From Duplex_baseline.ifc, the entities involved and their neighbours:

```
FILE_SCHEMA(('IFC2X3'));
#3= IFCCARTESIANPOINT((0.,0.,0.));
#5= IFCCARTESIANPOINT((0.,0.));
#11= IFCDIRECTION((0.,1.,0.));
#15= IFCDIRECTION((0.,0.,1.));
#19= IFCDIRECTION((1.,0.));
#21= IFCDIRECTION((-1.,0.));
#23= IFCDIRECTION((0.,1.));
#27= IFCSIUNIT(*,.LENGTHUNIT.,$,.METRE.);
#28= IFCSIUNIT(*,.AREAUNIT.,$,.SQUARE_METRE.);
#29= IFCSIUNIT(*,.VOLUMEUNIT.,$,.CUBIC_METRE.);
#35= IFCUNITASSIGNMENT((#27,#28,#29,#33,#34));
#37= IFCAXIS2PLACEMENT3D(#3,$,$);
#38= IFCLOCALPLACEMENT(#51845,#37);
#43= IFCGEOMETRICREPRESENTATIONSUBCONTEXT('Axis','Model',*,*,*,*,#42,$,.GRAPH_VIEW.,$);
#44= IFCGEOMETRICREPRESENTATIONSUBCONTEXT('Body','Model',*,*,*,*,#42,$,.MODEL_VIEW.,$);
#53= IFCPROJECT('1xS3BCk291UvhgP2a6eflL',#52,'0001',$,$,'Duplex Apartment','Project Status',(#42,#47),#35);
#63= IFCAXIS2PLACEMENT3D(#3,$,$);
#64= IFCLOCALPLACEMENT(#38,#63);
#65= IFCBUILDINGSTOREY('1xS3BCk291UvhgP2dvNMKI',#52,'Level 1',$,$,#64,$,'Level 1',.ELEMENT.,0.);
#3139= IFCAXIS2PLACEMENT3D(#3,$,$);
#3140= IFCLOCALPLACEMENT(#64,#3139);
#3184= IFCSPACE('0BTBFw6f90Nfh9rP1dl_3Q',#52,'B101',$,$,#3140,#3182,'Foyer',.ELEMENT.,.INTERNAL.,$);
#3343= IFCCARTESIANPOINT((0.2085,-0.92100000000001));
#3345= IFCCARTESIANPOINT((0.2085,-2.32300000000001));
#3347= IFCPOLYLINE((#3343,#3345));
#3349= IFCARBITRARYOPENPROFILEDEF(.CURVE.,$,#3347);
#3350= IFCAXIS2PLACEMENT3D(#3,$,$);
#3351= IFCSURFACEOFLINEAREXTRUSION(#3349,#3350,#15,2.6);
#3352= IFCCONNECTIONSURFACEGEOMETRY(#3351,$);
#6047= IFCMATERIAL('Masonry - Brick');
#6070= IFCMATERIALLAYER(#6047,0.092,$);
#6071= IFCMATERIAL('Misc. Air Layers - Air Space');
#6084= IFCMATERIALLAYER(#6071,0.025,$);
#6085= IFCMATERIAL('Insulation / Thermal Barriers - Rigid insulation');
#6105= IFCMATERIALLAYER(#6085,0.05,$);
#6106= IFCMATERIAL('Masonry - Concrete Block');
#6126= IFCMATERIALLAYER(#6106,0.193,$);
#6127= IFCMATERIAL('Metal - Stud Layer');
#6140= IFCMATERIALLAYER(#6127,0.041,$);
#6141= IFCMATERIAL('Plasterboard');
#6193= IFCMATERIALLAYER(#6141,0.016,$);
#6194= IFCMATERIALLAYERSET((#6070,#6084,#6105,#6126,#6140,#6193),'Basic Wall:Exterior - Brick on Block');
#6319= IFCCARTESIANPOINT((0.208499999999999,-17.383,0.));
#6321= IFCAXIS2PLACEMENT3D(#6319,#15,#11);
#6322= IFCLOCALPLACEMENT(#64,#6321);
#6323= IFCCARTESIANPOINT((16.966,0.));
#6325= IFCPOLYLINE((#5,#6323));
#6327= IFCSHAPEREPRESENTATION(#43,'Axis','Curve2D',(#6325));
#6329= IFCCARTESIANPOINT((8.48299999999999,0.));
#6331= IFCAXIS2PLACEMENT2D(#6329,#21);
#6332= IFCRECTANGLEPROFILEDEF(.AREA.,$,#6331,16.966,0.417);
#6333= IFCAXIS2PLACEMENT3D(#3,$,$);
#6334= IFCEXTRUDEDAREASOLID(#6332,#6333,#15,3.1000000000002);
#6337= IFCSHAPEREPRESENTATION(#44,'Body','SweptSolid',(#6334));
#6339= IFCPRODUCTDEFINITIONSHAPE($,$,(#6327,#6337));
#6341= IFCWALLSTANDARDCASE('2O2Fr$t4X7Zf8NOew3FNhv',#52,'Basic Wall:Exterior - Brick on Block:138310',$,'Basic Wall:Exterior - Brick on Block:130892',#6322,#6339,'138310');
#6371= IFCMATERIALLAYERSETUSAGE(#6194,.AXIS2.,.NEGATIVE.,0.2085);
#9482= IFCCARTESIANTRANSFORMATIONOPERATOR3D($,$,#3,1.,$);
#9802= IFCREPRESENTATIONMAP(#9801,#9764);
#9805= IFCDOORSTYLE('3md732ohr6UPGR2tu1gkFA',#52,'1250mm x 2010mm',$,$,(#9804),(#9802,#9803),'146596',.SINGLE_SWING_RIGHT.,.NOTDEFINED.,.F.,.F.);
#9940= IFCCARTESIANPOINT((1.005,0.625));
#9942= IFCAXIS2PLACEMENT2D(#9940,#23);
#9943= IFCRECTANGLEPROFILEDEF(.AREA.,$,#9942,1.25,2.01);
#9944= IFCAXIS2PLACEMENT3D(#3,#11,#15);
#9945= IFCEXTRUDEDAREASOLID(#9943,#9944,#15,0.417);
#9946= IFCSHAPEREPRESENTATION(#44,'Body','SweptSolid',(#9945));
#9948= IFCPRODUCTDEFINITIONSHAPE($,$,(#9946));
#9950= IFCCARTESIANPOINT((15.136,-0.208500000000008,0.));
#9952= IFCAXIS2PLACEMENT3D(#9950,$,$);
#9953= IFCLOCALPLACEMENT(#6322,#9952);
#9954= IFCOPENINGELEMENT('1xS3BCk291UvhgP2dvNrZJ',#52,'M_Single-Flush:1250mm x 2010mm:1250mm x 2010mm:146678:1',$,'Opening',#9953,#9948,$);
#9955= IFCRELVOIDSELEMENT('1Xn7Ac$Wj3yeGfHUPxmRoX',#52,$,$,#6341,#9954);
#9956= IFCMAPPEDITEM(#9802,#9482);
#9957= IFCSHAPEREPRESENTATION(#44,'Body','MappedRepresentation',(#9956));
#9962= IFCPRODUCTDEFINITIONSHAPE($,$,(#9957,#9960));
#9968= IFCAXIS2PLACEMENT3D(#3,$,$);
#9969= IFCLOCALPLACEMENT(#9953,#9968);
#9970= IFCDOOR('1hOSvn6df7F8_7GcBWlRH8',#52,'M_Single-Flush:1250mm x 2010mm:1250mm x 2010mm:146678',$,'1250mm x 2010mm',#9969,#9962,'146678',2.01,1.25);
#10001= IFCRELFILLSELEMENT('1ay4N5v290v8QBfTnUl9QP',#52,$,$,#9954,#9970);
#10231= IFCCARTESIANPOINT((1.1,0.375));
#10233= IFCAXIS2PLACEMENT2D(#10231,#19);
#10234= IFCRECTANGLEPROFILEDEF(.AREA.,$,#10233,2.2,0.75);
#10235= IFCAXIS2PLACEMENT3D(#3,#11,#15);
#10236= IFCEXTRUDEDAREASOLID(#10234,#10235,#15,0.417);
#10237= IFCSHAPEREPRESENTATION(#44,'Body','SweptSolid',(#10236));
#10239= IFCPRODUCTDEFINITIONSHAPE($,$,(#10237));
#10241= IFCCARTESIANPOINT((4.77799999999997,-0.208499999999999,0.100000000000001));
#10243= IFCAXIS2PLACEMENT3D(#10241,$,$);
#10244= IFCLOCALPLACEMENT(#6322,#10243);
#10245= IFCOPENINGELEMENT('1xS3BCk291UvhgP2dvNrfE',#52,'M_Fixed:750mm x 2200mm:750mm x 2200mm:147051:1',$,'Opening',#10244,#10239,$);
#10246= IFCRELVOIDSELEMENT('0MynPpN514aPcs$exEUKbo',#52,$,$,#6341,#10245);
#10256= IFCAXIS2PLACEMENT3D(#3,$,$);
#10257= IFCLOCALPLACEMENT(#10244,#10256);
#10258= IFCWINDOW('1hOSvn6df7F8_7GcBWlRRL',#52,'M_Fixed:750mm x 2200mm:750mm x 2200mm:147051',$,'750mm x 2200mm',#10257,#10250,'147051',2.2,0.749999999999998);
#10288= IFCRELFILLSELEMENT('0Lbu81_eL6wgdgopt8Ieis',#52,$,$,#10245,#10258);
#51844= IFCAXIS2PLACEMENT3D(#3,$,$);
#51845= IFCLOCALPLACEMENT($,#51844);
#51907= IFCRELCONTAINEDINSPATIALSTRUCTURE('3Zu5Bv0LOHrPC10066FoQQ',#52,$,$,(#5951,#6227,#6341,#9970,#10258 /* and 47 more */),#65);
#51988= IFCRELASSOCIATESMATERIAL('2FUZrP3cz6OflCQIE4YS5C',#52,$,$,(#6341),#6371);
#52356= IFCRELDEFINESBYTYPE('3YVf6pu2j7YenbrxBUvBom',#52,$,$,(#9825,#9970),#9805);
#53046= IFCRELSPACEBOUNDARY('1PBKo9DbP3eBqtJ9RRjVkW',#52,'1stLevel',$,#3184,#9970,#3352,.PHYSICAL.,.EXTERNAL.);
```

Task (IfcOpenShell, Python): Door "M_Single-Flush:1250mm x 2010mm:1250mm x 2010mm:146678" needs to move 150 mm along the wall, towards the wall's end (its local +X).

```python
import numpy as np
import ifcopenshell
import ifcopenshell.api.geometry
import ifcopenshell.util.placement
import ifcopenshell.util.unit

model = ifcopenshell.open("Duplex_baseline.ifc")
unit_scale = ifcopenshell.util.unit.calculate_unit_scale(model)

door = model.by_guid("1hOSvn6df7F8_7GcBWlRH8")
opening = door.FillsVoids[0].RelatingOpeningElement
wall = opening.VoidsElements[0].RelatingBuildingElement

wall_matrix = ifcopenshell.util.placement.get_local_placement(wall.ObjectPlacement)
shift = wall_matrix[:3, 0] * 0.15 / unit_scale
before = ifcopenshell.util.placement.get_local_placement(door.ObjectPlacement)[:3, 3].copy()

# The door is placed relative to its opening, so it follows when the opening moves.
matrix = ifcopenshell.util.placement.get_local_placement(opening.ObjectPlacement)
matrix[:3, 3] += shift
ifcopenshell.api.geometry.edit_object_placement(
    model, product=opening, matrix=matrix, is_si=False, should_transform_children=True
)

# Space boundary surfaces are stored in each space's coordinates; move them too.
for rel in door.ProvidesBoundaries:
    if not rel.ConnectionGeometry:
        continue
    surface = rel.ConnectionGeometry.SurfaceOnRelatingElement
    space_matrix = ifcopenshell.util.placement.get_local_placement(rel.RelatingSpace.ObjectPlacement)
    point = np.array(surface.Position.Location.Coordinates) + space_matrix[:3, :3].T @ shift
    surface.Position = model.createIfcAxis2Placement3D(
        model.createIfcCartesianPoint(point.tolist()), surface.Position.Axis, surface.Position.RefDirection
    )

after = ifcopenshell.util.placement.get_local_placement(door.ObjectPlacement)[:3, 3]
print("door moved by", (after - before).round(3) + 0.0)

model.write("Duplex_baseline_rev.ifc")
```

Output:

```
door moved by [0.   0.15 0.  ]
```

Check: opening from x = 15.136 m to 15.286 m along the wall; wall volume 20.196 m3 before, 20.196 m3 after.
